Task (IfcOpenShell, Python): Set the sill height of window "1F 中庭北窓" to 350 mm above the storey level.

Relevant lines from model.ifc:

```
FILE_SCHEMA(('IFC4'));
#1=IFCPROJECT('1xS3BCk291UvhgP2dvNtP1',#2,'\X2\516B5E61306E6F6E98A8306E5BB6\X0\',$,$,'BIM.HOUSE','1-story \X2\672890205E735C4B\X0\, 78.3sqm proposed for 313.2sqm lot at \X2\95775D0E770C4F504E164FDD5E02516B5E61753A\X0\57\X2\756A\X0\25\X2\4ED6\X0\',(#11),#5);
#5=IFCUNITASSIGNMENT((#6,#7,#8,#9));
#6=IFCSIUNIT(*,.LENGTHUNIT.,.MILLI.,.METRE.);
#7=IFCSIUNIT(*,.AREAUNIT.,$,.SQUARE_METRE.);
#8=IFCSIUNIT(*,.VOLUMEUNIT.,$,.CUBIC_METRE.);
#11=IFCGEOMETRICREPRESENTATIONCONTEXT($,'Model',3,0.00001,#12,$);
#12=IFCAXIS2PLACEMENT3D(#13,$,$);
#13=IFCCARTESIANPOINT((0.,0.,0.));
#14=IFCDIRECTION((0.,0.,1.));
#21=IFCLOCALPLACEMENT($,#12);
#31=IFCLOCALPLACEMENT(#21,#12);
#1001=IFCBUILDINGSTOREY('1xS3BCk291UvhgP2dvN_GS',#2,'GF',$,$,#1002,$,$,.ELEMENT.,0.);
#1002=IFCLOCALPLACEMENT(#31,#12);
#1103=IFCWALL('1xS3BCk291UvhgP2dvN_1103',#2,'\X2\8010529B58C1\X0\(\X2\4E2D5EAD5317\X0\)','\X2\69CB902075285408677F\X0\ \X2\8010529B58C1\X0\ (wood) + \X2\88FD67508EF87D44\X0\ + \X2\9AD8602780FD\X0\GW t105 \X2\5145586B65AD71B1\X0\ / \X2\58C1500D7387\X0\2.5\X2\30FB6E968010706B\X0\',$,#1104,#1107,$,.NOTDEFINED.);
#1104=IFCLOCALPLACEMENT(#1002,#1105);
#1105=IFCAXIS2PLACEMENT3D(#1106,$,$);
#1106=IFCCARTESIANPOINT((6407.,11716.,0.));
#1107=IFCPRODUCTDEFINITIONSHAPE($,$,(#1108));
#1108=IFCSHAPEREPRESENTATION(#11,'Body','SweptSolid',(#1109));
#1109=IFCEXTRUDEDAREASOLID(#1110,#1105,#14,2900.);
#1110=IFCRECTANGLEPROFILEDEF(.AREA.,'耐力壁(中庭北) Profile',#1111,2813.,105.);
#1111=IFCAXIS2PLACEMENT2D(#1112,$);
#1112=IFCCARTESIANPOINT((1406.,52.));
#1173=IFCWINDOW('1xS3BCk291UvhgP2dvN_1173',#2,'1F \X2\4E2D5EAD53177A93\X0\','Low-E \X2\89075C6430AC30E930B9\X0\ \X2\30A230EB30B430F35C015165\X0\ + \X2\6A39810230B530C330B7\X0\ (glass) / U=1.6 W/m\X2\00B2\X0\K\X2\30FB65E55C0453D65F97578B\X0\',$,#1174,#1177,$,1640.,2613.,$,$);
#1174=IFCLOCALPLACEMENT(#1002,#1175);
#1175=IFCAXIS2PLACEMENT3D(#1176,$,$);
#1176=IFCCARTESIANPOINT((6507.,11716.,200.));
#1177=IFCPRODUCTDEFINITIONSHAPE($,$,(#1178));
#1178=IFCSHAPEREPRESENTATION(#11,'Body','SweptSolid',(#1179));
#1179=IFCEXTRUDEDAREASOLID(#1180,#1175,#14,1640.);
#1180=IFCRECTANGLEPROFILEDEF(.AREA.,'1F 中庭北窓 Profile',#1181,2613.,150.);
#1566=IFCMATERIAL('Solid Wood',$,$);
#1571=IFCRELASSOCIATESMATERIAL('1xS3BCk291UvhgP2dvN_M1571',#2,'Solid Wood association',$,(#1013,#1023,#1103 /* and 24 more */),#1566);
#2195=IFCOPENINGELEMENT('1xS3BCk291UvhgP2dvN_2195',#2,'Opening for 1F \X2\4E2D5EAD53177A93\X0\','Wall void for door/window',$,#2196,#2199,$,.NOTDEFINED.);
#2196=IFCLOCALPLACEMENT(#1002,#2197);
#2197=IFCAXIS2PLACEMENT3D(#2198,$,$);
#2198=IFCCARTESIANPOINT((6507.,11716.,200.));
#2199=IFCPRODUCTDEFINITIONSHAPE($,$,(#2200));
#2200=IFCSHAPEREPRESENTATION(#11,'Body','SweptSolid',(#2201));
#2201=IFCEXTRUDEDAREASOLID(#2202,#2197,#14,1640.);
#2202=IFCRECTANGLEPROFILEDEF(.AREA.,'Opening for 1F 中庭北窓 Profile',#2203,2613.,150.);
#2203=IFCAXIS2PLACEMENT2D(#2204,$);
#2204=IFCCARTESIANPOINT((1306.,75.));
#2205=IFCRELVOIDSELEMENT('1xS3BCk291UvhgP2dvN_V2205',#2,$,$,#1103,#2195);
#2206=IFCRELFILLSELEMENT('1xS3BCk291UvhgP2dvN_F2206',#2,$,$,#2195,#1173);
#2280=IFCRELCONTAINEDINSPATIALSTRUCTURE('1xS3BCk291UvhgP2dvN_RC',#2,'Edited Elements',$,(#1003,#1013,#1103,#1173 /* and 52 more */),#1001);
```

```python
import numpy as np
import ifcopenshell
import ifcopenshell.api.geometry
import ifcopenshell.geom
import ifcopenshell.util.element
import ifcopenshell.util.placement
import ifcopenshell.util.shape
import ifcopenshell.util.unit

model = ifcopenshell.open("model.ifc")
unit_scale = ifcopenshell.util.unit.calculate_unit_scale(model)

window = model.by_guid("1xS3BCk291UvhgP2dvN_1173")
opening = window.FillsVoids[0].RelatingOpeningElement
storey = ifcopenshell.util.element.get_container(window, ifc_class="IfcBuildingStorey")
level = ifcopenshell.util.placement.get_local_placement(storey.ObjectPlacement)[2, 3]

# The opening's origin need not be at the sill, so measure its lowest point.
shape = ifcopenshell.geom.create_shape(ifcopenshell.geom.settings(), opening)
bottom = ifcopenshell.util.shape.get_shape_bottom_elevation(shape, shape.geometry) / unit_scale
dz = level + 350.0 - bottom

shift = np.array([0.0, 0.0, dz])
# The window is not placed relative to its opening, so move both.
for product in (opening, window):
    matrix = ifcopenshell.util.placement.get_local_placement(product.ObjectPlacement)
    matrix[:3, 3] += shift
    ifcopenshell.api.geometry.edit_object_placement(model, product=product, matrix=matrix, is_si=False)

print(f"moved by {dz * unit_scale:+.3f} m")

model.write("model_edited.ifc")
```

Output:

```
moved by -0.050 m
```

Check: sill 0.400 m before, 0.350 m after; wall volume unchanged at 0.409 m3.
